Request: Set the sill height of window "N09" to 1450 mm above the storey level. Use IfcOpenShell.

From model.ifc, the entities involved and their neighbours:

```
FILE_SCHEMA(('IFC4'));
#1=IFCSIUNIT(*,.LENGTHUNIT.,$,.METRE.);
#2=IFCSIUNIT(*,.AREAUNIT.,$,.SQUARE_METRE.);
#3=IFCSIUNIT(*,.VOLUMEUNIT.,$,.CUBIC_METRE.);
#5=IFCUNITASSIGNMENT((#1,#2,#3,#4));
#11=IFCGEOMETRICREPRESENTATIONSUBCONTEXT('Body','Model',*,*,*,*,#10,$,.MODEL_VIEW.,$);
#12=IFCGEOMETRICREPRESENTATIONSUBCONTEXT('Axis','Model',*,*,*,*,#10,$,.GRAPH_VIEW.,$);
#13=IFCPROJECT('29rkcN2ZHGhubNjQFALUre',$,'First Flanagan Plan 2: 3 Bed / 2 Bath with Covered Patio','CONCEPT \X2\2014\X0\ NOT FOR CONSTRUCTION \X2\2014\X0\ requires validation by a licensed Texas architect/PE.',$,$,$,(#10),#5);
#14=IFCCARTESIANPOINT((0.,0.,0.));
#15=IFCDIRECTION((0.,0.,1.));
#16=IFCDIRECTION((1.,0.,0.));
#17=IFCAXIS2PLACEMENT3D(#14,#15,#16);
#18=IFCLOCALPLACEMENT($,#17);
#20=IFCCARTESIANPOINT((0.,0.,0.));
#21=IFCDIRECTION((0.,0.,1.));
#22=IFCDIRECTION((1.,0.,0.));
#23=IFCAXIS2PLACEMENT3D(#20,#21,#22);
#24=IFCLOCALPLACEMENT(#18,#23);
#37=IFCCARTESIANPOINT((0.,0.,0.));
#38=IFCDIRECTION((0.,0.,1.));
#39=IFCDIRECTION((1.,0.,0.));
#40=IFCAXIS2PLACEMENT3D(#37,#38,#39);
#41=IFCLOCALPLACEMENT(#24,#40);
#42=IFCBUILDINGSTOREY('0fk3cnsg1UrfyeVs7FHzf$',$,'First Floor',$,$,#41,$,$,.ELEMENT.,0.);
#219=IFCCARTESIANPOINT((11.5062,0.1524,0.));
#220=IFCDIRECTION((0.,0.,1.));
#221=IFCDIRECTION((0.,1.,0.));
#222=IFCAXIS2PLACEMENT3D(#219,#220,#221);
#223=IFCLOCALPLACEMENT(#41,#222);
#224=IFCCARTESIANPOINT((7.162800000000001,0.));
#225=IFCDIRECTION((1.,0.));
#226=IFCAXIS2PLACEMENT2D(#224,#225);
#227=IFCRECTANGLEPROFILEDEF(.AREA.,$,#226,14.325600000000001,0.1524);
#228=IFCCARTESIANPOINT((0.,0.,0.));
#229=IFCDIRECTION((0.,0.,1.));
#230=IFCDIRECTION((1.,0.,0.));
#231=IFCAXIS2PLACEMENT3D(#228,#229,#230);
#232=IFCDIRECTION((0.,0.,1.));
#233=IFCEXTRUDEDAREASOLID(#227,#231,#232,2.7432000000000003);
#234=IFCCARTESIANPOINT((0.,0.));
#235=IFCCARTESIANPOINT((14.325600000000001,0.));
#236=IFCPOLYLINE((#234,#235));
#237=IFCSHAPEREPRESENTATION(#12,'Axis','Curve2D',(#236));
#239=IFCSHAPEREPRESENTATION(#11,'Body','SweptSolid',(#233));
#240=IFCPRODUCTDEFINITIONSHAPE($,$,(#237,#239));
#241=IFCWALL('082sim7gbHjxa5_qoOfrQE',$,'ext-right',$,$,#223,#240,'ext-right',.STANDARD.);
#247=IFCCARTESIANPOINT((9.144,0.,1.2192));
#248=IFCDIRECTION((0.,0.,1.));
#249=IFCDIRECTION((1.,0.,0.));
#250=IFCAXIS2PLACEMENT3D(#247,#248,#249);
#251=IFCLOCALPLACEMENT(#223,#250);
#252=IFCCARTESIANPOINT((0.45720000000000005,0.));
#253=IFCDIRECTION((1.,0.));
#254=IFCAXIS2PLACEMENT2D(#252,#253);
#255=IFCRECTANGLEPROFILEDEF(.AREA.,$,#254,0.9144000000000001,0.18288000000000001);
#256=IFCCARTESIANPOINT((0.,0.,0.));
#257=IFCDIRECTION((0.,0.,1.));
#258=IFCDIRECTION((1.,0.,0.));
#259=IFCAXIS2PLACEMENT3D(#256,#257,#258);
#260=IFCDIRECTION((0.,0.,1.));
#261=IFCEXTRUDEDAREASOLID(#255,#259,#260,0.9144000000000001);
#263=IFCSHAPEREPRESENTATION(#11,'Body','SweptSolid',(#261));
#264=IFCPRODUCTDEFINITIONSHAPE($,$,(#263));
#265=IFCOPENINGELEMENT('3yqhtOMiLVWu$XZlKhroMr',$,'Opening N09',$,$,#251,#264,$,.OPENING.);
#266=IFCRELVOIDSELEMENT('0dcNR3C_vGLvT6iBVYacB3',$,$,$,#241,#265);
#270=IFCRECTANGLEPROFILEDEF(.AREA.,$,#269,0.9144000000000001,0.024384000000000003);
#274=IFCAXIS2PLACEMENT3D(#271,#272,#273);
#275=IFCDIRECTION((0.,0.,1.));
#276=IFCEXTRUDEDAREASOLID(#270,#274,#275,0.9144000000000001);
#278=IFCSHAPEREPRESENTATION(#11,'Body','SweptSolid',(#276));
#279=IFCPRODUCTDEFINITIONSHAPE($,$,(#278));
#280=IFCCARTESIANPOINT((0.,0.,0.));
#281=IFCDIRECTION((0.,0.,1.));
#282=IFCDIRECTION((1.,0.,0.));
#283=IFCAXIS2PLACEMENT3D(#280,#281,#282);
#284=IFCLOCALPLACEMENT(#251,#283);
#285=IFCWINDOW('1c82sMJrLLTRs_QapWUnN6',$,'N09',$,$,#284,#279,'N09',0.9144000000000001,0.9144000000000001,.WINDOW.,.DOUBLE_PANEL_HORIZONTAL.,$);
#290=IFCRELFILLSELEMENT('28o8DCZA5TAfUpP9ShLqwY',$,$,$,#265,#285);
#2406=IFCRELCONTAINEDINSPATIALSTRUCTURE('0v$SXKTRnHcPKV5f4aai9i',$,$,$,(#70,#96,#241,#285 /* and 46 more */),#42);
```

```python
import numpy as np
import ifcopenshell
import ifcopenshell.api.geometry
import ifcopenshell.geom
import ifcopenshell.util.element
import ifcopenshell.util.placement
import ifcopenshell.util.shape
import ifcopenshell.util.unit

model = ifcopenshell.open("model.ifc")
unit_scale = ifcopenshell.util.unit.calculate_unit_scale(model)

window = model.by_id(285)
opening = window.FillsVoids[0].RelatingOpeningElement
storey = ifcopenshell.util.element.get_container(window, ifc_class="IfcBuildingStorey")
level = ifcopenshell.util.placement.get_local_placement(storey.ObjectPlacement)[2, 3]

# The opening's origin need not be at the sill, so measure its lowest point.
shape = ifcopenshell.geom.create_shape(ifcopenshell.geom.settings(), opening)
bottom = ifcopenshell.util.shape.get_shape_bottom_elevation(shape, shape.geometry) / unit_scale
dz = level + 1.45 - bottom

shift = np.array([0.0, 0.0, dz])
# The window is placed relative to its opening, so it follows when the opening moves.
matrix = ifcopenshell.util.placement.get_local_placement(opening.ObjectPlacement)
matrix[:3, 3] += shift
ifcopenshell.api.geometry.edit_object_placement(
    model, product=opening, matrix=matrix, is_si=False, should_transform_children=True
)

print(f"moved by {dz * unit_scale:+.3f} m")

model.write("model-out.ifc")
```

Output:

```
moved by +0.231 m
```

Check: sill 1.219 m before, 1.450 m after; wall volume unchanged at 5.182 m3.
